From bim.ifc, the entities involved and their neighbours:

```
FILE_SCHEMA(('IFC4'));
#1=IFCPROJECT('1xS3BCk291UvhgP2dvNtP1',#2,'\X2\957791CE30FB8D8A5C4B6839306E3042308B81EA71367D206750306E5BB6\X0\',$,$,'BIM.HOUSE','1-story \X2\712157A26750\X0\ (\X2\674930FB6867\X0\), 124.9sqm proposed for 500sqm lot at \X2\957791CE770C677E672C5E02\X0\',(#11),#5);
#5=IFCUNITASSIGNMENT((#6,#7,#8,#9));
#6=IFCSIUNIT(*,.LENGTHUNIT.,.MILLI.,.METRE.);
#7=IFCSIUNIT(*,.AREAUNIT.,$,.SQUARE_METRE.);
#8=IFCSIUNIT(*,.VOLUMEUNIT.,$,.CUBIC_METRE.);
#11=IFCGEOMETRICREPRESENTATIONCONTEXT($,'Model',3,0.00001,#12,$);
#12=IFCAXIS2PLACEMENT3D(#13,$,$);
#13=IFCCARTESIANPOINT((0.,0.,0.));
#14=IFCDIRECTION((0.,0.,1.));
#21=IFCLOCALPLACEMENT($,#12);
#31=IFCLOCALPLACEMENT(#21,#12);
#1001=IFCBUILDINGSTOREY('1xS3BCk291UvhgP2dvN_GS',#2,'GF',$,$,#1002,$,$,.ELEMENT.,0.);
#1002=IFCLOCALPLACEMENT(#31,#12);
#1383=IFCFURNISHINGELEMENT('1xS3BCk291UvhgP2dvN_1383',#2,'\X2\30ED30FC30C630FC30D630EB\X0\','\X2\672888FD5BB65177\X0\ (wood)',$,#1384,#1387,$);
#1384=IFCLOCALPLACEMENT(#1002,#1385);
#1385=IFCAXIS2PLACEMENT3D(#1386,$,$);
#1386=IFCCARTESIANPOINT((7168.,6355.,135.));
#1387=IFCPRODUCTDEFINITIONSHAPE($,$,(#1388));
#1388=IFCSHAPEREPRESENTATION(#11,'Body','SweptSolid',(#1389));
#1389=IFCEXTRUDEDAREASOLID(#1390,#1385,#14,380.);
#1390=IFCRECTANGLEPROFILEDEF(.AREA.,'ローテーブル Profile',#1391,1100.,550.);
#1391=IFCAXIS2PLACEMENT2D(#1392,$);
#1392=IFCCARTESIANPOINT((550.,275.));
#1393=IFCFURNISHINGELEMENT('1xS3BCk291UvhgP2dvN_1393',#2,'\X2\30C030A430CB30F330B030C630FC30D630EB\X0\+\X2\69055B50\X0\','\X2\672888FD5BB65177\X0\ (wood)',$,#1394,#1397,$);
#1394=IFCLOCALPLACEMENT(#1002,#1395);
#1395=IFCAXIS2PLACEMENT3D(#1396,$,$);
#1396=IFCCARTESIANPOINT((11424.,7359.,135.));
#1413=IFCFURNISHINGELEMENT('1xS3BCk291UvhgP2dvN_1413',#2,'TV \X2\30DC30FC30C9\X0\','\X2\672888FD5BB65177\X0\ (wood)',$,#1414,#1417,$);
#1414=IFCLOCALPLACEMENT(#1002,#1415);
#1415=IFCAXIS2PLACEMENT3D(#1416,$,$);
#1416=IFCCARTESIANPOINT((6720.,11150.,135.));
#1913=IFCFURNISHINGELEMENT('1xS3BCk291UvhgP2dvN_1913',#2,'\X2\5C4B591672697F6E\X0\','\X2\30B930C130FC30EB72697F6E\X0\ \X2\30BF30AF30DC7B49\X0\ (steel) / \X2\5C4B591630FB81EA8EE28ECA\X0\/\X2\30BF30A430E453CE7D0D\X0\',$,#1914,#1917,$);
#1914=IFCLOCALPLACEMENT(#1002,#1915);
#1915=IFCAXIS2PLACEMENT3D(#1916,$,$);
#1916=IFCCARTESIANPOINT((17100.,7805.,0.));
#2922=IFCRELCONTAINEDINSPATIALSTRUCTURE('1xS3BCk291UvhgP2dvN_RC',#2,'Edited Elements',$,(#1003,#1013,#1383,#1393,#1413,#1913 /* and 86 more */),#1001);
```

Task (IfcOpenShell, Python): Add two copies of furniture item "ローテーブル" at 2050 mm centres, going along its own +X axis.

```python
import ifcopenshell
import ifcopenshell.api.geometry
import ifcopenshell.api.root
import ifcopenshell.util.element
import ifcopenshell.util.placement
import ifcopenshell.util.unit

model = ifcopenshell.open("bim.ifc")
unit_scale = ifcopenshell.util.unit.calculate_unit_scale(model)


def reuse_history(source, copy):
    """copy_class also copies each property set's owner history, people and application; keep the originals."""
    for rel in copy.IsDefinedBy:
        if rel.is_a("IfcRelDefinesByProperties") and (history := rel.RelatingPropertyDefinition.OwnerHistory):
            rel.RelatingPropertyDefinition.OwnerHistory = source.OwnerHistory
            ifcopenshell.util.element.remove_deep2(model, history)


source = model.by_guid("1xS3BCk291UvhgP2dvN_1383")
base = ifcopenshell.util.placement.get_local_placement(source.ObjectPlacement)
step = base[:3, 0] * 2.05 / unit_scale

for i in range(1, 3):
    copy = ifcopenshell.api.root.copy_class(model, product=source)
    copy.Representation = ifcopenshell.util.element.copy_deep(
        model, source.Representation, exclude=["IfcGeometricRepresentationContext", "IfcRepresentationMap"]
    )
    reuse_history(source, copy)
    matrix = base.copy()
    matrix[:3, 3] += i * step
    print("added at", matrix[:3, 3].round(3) + 0.0)
    ifcopenshell.api.geometry.edit_object_placement(model, product=copy, matrix=matrix, is_si=False)

model.write("bim-out.ifc")
```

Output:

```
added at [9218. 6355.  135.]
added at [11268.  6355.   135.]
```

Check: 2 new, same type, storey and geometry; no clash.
